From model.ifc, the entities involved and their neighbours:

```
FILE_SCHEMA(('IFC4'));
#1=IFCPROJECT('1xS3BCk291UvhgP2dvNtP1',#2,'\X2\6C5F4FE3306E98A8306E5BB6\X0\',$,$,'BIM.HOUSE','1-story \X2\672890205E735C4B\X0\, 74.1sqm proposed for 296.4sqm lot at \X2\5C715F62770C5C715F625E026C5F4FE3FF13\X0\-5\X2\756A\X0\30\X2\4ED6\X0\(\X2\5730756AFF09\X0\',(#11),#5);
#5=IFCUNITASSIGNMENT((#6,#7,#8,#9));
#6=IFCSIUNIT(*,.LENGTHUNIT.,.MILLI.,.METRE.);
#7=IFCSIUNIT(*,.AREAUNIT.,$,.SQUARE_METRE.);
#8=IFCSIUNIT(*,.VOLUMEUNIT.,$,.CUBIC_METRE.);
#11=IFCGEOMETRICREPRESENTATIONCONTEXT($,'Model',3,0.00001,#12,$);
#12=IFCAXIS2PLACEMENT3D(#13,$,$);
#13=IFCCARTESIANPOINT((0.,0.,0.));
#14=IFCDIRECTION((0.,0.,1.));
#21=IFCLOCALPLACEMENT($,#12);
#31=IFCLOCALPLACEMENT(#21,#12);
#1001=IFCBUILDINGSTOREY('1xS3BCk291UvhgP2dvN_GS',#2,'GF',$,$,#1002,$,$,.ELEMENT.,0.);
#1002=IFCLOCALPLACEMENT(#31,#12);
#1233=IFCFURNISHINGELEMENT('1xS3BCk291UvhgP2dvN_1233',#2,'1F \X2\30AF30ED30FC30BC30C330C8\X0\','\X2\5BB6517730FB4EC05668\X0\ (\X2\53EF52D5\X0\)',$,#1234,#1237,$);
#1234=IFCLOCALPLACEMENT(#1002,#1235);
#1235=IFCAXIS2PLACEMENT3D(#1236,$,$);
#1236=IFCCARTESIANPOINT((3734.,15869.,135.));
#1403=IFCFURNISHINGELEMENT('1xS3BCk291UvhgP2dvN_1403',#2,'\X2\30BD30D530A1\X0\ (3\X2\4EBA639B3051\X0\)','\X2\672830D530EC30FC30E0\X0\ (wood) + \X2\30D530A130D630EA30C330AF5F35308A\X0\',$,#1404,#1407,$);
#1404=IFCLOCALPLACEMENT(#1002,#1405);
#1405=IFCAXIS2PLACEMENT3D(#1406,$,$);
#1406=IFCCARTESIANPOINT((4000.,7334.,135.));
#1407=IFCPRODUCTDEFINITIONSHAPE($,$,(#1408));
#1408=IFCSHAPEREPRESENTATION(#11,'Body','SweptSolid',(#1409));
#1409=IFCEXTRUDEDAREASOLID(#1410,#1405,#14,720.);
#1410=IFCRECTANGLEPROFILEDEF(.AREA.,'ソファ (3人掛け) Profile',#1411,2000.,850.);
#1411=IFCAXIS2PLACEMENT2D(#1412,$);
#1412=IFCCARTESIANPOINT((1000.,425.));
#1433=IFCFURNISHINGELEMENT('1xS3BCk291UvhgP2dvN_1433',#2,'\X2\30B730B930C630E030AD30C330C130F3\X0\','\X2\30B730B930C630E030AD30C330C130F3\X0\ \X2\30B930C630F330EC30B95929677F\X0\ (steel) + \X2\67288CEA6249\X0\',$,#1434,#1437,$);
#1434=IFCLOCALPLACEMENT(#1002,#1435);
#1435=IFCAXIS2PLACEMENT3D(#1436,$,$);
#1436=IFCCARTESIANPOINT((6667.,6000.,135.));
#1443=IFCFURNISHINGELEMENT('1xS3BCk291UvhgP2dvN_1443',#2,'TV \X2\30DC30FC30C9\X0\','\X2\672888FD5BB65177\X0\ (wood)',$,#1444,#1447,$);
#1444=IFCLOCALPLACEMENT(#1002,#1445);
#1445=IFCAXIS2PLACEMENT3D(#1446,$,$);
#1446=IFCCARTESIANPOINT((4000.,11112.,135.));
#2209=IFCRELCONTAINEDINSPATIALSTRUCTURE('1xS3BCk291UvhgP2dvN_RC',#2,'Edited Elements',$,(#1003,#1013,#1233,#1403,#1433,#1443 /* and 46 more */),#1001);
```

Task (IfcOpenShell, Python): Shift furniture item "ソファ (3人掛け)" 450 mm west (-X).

```python
import ifcopenshell
import ifcopenshell.api.geometry
import ifcopenshell.util.placement
import ifcopenshell.util.unit

model = ifcopenshell.open("model.ifc")
unit_scale = ifcopenshell.util.unit.calculate_unit_scale(model)

item = model.by_guid("1xS3BCk291UvhgP2dvN_1403")
matrix = ifcopenshell.util.placement.get_local_placement(item.ObjectPlacement)
matrix[0, 3] -= 0.45 / unit_scale
ifcopenshell.api.geometry.edit_object_placement(model, product=item, matrix=matrix, is_si=False)

print(ifcopenshell.util.placement.get_local_placement(item.ObjectPlacement).round(3) + 0.0)

model.write("model-out.ifc")
```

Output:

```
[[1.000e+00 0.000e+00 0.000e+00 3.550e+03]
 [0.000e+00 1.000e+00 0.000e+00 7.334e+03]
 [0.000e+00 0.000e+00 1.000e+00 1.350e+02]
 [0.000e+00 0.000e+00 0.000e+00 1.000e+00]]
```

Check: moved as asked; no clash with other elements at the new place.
